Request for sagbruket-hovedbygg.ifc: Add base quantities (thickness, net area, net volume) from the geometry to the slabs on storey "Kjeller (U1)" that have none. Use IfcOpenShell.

First a look at what the model holds.

```python
import ifcopenshell
import ifcopenshell.util.element
import ifcopenshell.util.unit

model = ifcopenshell.open("sagbruket-hovedbygg.ifc")
print(model.schema)
for unit_type in ("LENGTHUNIT", "AREAUNIT", "VOLUMEUNIT"):
    print(unit_type, ifcopenshell.util.unit.calculate_unit_scale(model, unit_type))
storey = next(s for s in model.by_type("IfcBuildingStorey") if s.Name == "Kjeller (U1)")
slabs = [e for e in ifcopenshell.util.element.get_decomposition(storey) if e.is_a("IfcSlab")]
for e in sorted(slabs, key=lambda e: e.id()):
    print(e.id(), e.is_a(), e.Name, list(ifcopenshell.util.element.get_psets(e, qtos_only=True)), sep=" | ")
```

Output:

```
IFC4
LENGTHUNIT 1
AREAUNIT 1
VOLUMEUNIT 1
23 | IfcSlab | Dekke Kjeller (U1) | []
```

```python
import ifcopenshell
import ifcopenshell.api.pset
import ifcopenshell.geom
import ifcopenshell.util.element
import ifcopenshell.util.shape
import ifcopenshell.util.unit

model = ifcopenshell.open("sagbruket-hovedbygg.ifc")
unit_scale = ifcopenshell.util.unit.calculate_unit_scale(model)
area_scale = ifcopenshell.util.unit.calculate_unit_scale(model, "AREAUNIT")
volume_scale = ifcopenshell.util.unit.calculate_unit_scale(model, "VOLUMEUNIT")
settings = ifcopenshell.geom.settings()

storey = next(s for s in model.by_type("IfcBuildingStorey") if s.Name == "Kjeller (U1)")
slabs = [e for e in ifcopenshell.util.element.get_decomposition(storey) if e.is_a("IfcSlab")]

for e in sorted(slabs, key=lambda e: e.id()):
    if ifcopenshell.util.element.get_psets(e, qtos_only=True, should_inherit=False):
        continue
    # Geometry comes back in metres, in the element's own axes.
    shape = ifcopenshell.geom.create_shape(settings, e)
    values = {
        "Width": ifcopenshell.util.shape.get_z(shape.geometry) / unit_scale,
        "NetArea": ifcopenshell.util.shape.get_footprint_area(shape.geometry) / area_scale,
        "NetVolume": ifcopenshell.util.shape.get_volume(shape.geometry) / volume_scale,
    }
    qto = ifcopenshell.api.pset.add_qto(model, product=e, name="Qto_SlabBaseQuantities")
    ifcopenshell.api.pset.edit_qto(model, qto=qto, properties=values)
    print(e.id(), {k: round(v, 3) for k, v in values.items()})

model.write("sagbruket-hovedbygg-out.ifc")
```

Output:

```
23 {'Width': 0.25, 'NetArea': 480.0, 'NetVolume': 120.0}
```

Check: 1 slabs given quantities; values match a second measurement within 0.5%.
